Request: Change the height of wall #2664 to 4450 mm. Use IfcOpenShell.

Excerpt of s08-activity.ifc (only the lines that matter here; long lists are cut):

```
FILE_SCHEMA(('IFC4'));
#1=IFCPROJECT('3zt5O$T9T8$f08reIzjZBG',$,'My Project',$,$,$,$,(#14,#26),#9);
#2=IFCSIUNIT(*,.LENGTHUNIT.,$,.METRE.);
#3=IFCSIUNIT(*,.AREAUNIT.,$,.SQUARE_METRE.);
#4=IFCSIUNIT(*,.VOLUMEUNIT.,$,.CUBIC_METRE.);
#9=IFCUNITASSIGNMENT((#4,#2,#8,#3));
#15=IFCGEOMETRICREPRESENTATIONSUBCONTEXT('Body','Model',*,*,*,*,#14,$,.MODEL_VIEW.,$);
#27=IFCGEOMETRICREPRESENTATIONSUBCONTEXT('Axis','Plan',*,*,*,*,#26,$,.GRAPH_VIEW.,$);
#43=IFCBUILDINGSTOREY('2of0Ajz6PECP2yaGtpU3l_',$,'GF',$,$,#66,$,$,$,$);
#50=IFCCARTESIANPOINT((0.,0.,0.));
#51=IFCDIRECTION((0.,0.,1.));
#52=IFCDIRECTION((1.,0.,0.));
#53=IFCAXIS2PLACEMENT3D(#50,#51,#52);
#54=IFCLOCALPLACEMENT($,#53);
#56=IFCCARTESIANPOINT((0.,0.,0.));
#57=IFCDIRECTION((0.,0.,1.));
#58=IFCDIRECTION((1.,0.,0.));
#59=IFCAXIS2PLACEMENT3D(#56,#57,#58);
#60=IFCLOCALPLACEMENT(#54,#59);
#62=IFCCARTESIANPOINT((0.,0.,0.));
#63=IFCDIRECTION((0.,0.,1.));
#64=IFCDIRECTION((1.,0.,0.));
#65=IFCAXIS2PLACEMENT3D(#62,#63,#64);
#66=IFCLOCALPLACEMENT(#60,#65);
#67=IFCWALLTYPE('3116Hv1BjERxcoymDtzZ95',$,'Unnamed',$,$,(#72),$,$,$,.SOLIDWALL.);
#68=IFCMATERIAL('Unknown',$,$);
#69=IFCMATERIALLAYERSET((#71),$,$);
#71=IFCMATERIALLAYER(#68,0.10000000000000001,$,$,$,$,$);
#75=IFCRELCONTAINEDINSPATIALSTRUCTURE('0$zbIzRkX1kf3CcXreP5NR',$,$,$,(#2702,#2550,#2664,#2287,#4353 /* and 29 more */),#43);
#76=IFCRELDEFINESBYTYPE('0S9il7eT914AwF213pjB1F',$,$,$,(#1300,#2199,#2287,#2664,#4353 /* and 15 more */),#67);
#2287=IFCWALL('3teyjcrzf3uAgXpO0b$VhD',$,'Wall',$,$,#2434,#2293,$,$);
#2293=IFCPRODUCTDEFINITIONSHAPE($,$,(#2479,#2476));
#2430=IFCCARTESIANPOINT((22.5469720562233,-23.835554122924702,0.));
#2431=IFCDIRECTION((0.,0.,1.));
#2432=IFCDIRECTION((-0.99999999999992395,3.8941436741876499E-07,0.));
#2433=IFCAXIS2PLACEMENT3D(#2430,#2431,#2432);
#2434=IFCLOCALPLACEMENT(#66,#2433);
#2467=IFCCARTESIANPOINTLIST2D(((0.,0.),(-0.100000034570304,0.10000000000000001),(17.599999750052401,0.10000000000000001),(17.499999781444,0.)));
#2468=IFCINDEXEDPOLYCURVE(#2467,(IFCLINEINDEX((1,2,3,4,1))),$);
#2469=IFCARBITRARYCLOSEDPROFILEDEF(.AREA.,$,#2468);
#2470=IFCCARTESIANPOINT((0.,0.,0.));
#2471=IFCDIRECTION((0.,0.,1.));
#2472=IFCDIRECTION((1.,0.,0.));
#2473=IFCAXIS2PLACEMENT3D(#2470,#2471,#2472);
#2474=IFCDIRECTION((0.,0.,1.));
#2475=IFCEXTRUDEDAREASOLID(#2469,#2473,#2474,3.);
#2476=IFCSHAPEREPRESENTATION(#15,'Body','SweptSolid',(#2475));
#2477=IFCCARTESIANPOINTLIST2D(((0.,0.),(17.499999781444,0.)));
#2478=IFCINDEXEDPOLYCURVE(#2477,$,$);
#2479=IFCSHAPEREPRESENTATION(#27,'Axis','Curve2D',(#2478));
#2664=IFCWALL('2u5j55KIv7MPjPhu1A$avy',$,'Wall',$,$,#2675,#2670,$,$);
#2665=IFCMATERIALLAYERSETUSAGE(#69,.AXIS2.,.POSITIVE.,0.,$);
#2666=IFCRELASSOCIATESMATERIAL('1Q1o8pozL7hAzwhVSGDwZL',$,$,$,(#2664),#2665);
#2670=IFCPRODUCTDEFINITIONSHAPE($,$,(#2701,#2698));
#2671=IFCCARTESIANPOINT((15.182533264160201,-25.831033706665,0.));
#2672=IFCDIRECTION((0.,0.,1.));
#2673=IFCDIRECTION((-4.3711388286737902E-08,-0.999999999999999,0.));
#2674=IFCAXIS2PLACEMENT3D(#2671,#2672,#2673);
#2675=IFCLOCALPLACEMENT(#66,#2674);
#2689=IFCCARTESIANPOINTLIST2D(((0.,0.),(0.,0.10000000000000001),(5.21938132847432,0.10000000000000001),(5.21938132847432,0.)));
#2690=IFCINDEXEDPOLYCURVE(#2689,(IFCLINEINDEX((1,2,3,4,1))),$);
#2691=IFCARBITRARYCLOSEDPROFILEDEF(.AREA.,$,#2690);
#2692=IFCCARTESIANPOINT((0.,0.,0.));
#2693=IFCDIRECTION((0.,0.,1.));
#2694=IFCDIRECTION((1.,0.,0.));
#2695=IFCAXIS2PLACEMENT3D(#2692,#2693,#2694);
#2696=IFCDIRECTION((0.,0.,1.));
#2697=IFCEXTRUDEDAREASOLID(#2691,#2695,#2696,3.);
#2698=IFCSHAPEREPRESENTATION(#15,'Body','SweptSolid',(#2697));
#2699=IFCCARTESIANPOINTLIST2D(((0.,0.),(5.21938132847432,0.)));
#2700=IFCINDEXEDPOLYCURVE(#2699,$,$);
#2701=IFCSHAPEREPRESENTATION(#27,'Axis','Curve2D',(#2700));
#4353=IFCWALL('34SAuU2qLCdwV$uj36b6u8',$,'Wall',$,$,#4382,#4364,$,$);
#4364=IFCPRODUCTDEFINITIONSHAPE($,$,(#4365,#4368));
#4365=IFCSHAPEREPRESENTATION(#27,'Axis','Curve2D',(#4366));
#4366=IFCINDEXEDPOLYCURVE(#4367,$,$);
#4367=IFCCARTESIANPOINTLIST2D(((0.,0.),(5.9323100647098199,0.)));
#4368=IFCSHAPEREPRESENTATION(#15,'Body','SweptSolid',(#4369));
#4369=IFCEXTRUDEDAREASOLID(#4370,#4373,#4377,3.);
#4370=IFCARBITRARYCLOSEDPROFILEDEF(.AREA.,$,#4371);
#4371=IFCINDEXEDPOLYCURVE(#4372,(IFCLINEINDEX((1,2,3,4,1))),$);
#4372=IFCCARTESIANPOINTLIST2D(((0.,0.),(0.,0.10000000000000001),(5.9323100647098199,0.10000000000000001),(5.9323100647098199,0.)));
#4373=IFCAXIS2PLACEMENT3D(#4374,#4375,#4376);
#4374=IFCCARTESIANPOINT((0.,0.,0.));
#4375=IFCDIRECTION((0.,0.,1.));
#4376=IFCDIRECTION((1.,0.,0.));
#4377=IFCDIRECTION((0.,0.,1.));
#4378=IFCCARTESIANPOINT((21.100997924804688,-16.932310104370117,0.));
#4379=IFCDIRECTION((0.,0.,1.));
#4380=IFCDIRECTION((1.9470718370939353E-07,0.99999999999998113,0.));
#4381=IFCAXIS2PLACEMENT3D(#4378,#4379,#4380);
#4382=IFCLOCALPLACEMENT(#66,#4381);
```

```python
import ifcopenshell
import ifcopenshell.geom
import ifcopenshell.util.representation
import ifcopenshell.util.shape

model = ifcopenshell.open("s08-activity.ifc")
settings = ifcopenshell.geom.settings()


def volume(element):
    """Net volume in cubic metres, openings subtracted."""
    shape = ifcopenshell.geom.create_shape(settings, element)
    return ifcopenshell.util.shape.get_volume(shape.geometry)


wall = model.by_guid("2u5j55KIv7MPjPhu1A$avy")
before = volume(wall)

body = ifcopenshell.util.representation.get_representation(wall, "Model", "Body")
solid = body.Items[0]
old_height = solid.Depth
solid.Depth = 4.45
after = volume(wall)

print(f"height {old_height:g} -> {solid.Depth:g}, volume {before:.3f} -> {after:.3f} m3")

model.write("s08-activity_edited.ifc")
```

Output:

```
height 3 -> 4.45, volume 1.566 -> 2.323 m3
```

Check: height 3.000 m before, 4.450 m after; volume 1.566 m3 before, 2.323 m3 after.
